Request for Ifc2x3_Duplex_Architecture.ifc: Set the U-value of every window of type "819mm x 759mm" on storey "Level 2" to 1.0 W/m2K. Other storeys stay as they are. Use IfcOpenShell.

First a look at what the model holds.

```python
import ifcopenshell
import ifcopenshell.util.element

model = ifcopenshell.open("Ifc2x3_Duplex_Architecture.ifc")
print(model.schema)
storey = next(s for s in model.by_type("IfcBuildingStorey") if s.Name == "Level 2")
windows = [e for e in ifcopenshell.util.element.get_decomposition(storey) if e.is_a("IfcWindow")]
seen = {}
for e in windows:
    element_type = ifcopenshell.util.element.get_type(e)
    key = (element_type.Name if element_type != e and element_type else None, ifcopenshell.util.element.get_pset(e, "Pset_WindowCommon", "ThermalTransmittance"))
    seen[key] = seen.get(key, 0) + 1
for (name, value), count in sorted(seen.items(), key=str):
    print(count, "x", name, "|", value)
```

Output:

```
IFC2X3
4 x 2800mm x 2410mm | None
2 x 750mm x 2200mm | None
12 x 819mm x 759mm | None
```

```python
import ifcopenshell
import ifcopenshell.api.pset
import ifcopenshell.util.element

model = ifcopenshell.open("Ifc2x3_Duplex_Architecture.ifc")

storey = next(s for s in model.by_type("IfcBuildingStorey") if s.Name == "Level 2")
windows = [e for e in ifcopenshell.util.element.get_decomposition(storey) if e.is_a("IfcWindow")]

count = 0
for e in windows:
    element_type = ifcopenshell.util.element.get_type(e)
    if element_type in (None, e) or element_type.Name != "819mm x 759mm":
        continue
    # add_pset returns the element's existing set when there is one.
    pset = ifcopenshell.api.pset.add_pset(model, product=e, name="Pset_WindowCommon")
    ifcopenshell.api.pset.edit_pset(model, pset=pset, properties={"ThermalTransmittance": 1.0})
    count += 1

print(count, "windows updated")

model.write("Ifc2x3_Duplex_Architecture_updated.ifc")
```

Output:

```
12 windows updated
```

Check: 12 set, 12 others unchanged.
